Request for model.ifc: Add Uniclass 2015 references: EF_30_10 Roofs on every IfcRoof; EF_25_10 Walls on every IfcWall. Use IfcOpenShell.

First a look at what the model holds.

```python
import ifcopenshell

model = ifcopenshell.open("model.ifc")
print(model.schema)
print("classifications:", [c.Name for c in model.by_type("IfcClassification")])
for ifc_class in ("IfcDoor", "IfcRoof", "IfcStair", "IfcWall", "IfcWindow"):
    print(ifc_class, len(model.by_type(ifc_class)))
```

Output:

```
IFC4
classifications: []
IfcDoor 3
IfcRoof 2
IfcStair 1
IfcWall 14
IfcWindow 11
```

```python
import ifcopenshell
import ifcopenshell.api.classification

model = ifcopenshell.open("model.ifc")

system = ifcopenshell.api.classification.add_classification(model, classification="Uniclass 2015")

codes = {
    "IfcRoof": ("EF_30_10", "Roofs"),
    "IfcWall": ("EF_25_10", "Walls"),
}
for ifc_class, (code, name) in codes.items():
    products = model.by_type(ifc_class)
    ifcopenshell.api.classification.add_reference(
        model, products=products, classification=system, identification=code, name=name
    )
    print(code, len(products))

model.write("model_v2.ifc")
```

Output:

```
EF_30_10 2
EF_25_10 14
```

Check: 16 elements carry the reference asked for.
